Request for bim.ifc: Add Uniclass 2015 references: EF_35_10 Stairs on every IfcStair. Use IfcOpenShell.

First a look at what the model holds.

```python
import ifcopenshell

model = ifcopenshell.open("bim.ifc")
print(model.schema)
print("classifications:", [c.Name for c in model.by_type("IfcClassification")])
for ifc_class in ("IfcDoor", "IfcRoof", "IfcStair", "IfcWall", "IfcWindow"):
    print(ifc_class, len(model.by_type(ifc_class)))
```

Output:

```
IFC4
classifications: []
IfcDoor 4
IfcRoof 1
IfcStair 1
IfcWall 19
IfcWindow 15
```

```python
import ifcopenshell
import ifcopenshell.api.classification

model = ifcopenshell.open("bim.ifc")

system = ifcopenshell.api.classification.add_classification(model, classification="Uniclass 2015")

codes = {
    "IfcStair": ("EF_35_10", "Stairs"),
}
for ifc_class, (code, name) in codes.items():
    products = model.by_type(ifc_class)
    ifcopenshell.api.classification.add_reference(
        model, products=products, classification=system, identification=code, name=name
    )
    print(code, len(products))

model.write("bim_rev.ifc")
```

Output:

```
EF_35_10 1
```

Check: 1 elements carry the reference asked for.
